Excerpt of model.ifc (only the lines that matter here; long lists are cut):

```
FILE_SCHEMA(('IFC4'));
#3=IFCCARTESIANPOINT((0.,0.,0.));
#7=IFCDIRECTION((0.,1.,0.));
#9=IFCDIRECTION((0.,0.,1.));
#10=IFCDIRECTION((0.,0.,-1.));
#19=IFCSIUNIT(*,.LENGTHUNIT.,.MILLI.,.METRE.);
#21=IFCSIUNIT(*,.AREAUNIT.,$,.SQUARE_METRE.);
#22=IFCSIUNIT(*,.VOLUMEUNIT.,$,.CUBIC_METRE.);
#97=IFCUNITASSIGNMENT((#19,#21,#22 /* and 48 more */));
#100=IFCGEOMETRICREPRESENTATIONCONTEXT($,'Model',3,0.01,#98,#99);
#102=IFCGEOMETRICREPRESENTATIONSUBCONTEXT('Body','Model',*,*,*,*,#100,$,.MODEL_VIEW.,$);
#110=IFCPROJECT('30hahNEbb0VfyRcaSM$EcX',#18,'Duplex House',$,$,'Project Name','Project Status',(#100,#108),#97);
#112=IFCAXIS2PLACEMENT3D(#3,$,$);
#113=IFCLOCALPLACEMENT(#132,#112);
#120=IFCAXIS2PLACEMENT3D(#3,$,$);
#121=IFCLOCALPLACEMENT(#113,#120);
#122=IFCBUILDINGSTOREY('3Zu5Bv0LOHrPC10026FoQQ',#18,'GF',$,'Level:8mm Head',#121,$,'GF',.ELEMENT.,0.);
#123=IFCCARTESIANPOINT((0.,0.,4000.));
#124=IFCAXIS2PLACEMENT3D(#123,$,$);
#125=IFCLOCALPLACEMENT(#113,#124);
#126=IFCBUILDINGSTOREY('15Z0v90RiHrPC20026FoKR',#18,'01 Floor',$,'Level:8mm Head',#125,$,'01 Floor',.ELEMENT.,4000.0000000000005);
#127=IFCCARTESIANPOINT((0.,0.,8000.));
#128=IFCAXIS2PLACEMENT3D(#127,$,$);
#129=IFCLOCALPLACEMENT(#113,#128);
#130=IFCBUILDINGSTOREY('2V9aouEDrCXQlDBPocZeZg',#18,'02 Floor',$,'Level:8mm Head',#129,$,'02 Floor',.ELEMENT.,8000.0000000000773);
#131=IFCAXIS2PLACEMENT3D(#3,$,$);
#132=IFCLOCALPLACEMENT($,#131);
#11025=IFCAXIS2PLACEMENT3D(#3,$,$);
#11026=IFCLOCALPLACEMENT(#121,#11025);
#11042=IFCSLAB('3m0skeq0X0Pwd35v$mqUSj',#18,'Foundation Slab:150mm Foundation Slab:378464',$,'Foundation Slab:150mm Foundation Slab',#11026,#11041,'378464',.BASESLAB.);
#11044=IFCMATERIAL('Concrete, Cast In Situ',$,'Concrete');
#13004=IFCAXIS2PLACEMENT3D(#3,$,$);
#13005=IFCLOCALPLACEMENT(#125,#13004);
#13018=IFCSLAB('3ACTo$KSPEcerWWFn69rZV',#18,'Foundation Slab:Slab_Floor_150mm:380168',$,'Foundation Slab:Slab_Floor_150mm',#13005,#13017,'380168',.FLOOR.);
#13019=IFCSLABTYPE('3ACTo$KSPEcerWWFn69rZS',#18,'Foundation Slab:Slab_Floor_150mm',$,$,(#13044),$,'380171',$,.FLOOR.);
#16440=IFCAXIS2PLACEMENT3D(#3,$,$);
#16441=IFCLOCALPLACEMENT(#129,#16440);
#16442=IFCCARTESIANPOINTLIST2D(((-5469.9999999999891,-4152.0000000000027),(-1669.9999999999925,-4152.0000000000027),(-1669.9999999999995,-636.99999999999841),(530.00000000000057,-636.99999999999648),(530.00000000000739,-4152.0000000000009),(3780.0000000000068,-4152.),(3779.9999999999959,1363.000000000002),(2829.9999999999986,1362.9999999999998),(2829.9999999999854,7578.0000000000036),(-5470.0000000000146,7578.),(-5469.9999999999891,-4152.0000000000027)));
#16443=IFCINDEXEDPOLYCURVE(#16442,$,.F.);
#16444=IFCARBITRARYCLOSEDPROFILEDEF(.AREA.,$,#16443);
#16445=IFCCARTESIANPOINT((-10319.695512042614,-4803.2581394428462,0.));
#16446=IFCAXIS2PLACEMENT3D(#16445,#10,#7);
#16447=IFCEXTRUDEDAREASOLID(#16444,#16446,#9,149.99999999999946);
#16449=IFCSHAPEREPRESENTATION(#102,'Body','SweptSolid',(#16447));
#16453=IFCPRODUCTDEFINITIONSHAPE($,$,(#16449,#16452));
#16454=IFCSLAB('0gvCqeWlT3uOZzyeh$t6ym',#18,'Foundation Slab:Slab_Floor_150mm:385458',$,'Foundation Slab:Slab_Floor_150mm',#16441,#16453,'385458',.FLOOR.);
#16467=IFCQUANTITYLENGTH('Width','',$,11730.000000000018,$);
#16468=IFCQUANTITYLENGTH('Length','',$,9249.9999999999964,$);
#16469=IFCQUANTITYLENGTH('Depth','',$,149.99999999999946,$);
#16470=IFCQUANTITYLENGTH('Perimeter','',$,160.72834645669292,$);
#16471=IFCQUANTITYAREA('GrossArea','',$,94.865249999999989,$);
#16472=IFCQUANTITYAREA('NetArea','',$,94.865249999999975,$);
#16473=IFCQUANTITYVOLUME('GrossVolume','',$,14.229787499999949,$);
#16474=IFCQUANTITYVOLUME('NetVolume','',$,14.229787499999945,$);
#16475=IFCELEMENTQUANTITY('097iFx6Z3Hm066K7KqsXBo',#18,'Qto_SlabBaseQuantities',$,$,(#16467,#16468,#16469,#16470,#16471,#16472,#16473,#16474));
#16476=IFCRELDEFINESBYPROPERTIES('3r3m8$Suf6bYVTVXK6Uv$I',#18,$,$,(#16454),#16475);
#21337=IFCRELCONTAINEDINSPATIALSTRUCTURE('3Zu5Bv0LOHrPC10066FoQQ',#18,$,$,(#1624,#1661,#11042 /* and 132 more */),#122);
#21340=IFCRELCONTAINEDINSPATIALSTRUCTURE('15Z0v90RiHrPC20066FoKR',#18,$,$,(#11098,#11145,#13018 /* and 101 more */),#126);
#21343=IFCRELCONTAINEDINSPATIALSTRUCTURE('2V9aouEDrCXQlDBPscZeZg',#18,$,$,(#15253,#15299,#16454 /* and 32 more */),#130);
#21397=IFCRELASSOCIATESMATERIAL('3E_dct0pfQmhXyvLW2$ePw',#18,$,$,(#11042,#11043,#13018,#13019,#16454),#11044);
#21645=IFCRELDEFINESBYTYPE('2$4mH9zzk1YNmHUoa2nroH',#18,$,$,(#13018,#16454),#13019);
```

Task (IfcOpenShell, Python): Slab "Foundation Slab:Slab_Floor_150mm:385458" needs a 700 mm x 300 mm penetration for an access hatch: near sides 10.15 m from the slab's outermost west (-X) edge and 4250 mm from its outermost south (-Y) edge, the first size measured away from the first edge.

```python
import numpy as np
import ifcopenshell
import ifcopenshell.api.feature
import ifcopenshell.api.geometry
import ifcopenshell.api.pset
import ifcopenshell.api.root
import ifcopenshell.geom
import ifcopenshell.util.element
import ifcopenshell.util.placement
import ifcopenshell.util.representation
import ifcopenshell.util.shape
import ifcopenshell.util.unit

model = ifcopenshell.open("model.ifc")
unit_scale = ifcopenshell.util.unit.calculate_unit_scale(model)
area_scale = ifcopenshell.util.unit.calculate_unit_scale(model, "AREAUNIT")
volume_scale = ifcopenshell.util.unit.calculate_unit_scale(model, "VOLUMEUNIT")
settings = ifcopenshell.geom.settings()


def volume(element):
    """Net volume in cubic metres, openings subtracted."""
    shape = ifcopenshell.geom.create_shape(settings, element)
    return ifcopenshell.util.shape.get_volume(shape.geometry)


slab = model.by_guid("0gvCqeWlT3uOZzyeh$t6ym")
before = volume(slab)

# Extent in the slab's own axes, in metres. The edges named are its -X and -Y sides.
slab_shape = ifcopenshell.geom.create_shape(settings, slab)
vertices = ifcopenshell.util.shape.get_vertices(slab_shape.geometry)
x_min, y_min, bottom = vertices.min(axis=0)
top = vertices[:, 2].max()

opening = ifcopenshell.api.root.create_entity(model, ifc_class="IfcOpeningElement", name="Access hatch opening", predefined_type="OPENING")
context = ifcopenshell.util.representation.get_context(model, "Model", "Body", "MODEL_VIEW")
width, depth = 0.7, 0.3
outline = [(0.0, 0.0), (width, 0.0), (width, depth), (0.0, depth), (0.0, 0.0)]
# Overshoot both faces by 50 mm so the cut is clean.
shape = ifcopenshell.api.geometry.add_slab_representation(
    model, context=context, depth=top - bottom + 0.1, polyline=outline
)
ifcopenshell.api.geometry.assign_representation(model, product=opening, representation=shape)

matrix = ifcopenshell.util.placement.get_local_placement(slab.ObjectPlacement)
matrix[:, 3] = matrix @ np.append(np.array([x_min + 10.15, y_min + 4.25, bottom - 0.05]) / unit_scale, 1.0)
ifcopenshell.api.geometry.edit_object_placement(model, product=opening, matrix=matrix, is_si=False)
ifcopenshell.api.feature.add_feature(model, feature=opening, element=slab)

after = volume(slab)

# Update the slab's stored quantities.
qto = model.by_id(ifcopenshell.util.element.get_pset(slab, "Qto_SlabBaseQuantities", should_inherit=False)["id"])
ifcopenshell.api.pset.edit_qto(model, qto=qto, properties={
    "NetArea": after / (top - bottom) / area_scale,
    "NetVolume": after / volume_scale,
})

print(f"slab volume {before:.3f} -> {after:.3f} m3")

model.write("model_edited.ifc")
```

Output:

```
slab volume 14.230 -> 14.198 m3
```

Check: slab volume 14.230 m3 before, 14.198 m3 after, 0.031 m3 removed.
